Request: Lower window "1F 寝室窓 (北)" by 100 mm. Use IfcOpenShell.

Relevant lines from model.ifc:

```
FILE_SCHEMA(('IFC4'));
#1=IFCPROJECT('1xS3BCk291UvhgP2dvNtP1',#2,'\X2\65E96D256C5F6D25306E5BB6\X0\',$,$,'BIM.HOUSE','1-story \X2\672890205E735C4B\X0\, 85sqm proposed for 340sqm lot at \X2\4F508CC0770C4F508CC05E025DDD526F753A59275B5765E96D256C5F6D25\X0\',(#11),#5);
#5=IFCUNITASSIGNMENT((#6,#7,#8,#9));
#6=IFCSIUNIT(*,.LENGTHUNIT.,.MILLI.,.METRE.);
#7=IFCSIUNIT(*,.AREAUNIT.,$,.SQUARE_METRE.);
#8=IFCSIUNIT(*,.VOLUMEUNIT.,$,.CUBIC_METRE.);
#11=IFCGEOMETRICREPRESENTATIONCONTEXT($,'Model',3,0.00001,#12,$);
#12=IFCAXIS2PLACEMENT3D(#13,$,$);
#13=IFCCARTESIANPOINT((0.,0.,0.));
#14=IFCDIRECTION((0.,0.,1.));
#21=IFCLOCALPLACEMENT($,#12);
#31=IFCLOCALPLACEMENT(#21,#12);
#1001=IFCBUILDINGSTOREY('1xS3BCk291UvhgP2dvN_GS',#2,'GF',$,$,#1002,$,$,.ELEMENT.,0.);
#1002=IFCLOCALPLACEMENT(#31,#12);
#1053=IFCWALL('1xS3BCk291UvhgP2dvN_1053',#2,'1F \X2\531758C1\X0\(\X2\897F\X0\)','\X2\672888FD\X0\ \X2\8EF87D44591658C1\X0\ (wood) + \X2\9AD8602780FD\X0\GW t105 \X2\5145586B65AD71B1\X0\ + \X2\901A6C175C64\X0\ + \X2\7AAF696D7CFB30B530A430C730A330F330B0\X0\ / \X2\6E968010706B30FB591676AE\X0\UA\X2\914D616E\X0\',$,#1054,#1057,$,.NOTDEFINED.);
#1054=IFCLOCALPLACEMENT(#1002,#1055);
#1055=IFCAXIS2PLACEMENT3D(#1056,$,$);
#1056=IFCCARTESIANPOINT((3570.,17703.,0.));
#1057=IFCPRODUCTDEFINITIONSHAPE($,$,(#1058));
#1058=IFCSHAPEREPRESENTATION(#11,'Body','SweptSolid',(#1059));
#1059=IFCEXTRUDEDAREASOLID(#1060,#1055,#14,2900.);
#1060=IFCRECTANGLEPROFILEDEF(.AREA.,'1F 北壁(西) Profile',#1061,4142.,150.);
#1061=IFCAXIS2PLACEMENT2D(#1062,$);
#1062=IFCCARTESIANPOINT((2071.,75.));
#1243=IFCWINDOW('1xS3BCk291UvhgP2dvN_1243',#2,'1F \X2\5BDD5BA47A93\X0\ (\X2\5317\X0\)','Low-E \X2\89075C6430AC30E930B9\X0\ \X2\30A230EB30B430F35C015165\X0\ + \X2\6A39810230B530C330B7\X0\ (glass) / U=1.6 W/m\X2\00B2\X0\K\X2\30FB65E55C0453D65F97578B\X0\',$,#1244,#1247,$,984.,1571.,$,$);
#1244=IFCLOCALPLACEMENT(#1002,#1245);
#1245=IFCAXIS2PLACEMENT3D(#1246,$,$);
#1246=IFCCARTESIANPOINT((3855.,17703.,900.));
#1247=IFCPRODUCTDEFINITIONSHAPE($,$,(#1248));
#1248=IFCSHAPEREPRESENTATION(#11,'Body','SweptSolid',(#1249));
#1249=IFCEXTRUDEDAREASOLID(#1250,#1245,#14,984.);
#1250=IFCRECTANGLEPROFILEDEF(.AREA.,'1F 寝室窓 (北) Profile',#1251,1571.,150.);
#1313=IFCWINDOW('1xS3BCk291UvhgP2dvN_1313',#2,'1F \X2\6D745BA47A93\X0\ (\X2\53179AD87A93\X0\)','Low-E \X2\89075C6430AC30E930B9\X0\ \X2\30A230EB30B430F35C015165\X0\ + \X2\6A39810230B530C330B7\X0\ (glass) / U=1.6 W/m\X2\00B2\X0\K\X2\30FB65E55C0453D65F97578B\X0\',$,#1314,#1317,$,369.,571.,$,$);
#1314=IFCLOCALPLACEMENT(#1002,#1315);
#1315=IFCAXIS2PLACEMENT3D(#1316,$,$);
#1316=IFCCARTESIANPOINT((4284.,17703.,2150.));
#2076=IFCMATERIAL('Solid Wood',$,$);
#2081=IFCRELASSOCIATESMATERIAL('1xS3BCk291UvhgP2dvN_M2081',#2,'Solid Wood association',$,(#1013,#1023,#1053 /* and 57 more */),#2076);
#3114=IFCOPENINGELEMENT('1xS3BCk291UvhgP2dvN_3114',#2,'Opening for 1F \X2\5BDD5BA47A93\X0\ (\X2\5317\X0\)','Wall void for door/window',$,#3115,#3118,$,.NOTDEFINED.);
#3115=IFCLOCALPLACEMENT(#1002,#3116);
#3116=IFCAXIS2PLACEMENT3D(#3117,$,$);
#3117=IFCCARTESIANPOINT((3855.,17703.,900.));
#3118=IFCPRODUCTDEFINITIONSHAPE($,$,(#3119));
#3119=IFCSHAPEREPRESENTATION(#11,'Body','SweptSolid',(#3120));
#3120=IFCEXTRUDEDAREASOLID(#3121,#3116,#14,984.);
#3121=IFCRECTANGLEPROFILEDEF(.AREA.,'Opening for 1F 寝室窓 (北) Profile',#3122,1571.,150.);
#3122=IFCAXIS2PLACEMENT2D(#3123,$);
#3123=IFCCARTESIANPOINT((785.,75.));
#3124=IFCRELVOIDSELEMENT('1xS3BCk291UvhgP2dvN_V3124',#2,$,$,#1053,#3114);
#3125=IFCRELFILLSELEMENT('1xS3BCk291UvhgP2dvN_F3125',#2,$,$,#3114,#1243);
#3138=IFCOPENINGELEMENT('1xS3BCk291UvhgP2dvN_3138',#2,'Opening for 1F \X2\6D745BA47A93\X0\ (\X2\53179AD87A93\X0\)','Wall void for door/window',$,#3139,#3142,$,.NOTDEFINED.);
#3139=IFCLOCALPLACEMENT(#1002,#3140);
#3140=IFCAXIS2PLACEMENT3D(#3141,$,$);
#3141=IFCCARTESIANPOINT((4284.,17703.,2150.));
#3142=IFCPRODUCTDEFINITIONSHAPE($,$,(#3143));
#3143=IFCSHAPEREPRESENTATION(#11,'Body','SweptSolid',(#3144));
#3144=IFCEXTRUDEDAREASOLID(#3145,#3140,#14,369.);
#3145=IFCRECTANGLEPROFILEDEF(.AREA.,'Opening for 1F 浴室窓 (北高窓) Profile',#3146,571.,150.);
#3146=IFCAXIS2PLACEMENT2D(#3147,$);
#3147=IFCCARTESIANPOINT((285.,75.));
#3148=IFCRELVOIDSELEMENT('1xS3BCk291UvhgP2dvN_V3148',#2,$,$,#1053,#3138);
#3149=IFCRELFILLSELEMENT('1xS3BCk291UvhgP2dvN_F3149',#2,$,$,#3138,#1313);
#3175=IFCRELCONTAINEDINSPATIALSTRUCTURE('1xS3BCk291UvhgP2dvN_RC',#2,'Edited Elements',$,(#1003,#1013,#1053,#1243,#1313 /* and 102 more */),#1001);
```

```python
import numpy as np
import ifcopenshell
import ifcopenshell.api.geometry
import ifcopenshell.util.placement
import ifcopenshell.util.unit

model = ifcopenshell.open("model.ifc")
unit_scale = ifcopenshell.util.unit.calculate_unit_scale(model)

window = model.by_guid("1xS3BCk291UvhgP2dvN_1243")
opening = window.FillsVoids[0].RelatingOpeningElement
dz = -0.1 / unit_scale

shift = np.array([0.0, 0.0, dz])
# The window is not placed relative to its opening, so move both.
for product in (opening, window):
    matrix = ifcopenshell.util.placement.get_local_placement(product.ObjectPlacement)
    matrix[:3, 3] += shift
    ifcopenshell.api.geometry.edit_object_placement(model, product=product, matrix=matrix, is_si=False)

print(f"moved by {dz * unit_scale:+.3f} m")

model.write("model_rev.ifc")
```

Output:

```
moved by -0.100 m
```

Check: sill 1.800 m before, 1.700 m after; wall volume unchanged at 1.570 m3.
